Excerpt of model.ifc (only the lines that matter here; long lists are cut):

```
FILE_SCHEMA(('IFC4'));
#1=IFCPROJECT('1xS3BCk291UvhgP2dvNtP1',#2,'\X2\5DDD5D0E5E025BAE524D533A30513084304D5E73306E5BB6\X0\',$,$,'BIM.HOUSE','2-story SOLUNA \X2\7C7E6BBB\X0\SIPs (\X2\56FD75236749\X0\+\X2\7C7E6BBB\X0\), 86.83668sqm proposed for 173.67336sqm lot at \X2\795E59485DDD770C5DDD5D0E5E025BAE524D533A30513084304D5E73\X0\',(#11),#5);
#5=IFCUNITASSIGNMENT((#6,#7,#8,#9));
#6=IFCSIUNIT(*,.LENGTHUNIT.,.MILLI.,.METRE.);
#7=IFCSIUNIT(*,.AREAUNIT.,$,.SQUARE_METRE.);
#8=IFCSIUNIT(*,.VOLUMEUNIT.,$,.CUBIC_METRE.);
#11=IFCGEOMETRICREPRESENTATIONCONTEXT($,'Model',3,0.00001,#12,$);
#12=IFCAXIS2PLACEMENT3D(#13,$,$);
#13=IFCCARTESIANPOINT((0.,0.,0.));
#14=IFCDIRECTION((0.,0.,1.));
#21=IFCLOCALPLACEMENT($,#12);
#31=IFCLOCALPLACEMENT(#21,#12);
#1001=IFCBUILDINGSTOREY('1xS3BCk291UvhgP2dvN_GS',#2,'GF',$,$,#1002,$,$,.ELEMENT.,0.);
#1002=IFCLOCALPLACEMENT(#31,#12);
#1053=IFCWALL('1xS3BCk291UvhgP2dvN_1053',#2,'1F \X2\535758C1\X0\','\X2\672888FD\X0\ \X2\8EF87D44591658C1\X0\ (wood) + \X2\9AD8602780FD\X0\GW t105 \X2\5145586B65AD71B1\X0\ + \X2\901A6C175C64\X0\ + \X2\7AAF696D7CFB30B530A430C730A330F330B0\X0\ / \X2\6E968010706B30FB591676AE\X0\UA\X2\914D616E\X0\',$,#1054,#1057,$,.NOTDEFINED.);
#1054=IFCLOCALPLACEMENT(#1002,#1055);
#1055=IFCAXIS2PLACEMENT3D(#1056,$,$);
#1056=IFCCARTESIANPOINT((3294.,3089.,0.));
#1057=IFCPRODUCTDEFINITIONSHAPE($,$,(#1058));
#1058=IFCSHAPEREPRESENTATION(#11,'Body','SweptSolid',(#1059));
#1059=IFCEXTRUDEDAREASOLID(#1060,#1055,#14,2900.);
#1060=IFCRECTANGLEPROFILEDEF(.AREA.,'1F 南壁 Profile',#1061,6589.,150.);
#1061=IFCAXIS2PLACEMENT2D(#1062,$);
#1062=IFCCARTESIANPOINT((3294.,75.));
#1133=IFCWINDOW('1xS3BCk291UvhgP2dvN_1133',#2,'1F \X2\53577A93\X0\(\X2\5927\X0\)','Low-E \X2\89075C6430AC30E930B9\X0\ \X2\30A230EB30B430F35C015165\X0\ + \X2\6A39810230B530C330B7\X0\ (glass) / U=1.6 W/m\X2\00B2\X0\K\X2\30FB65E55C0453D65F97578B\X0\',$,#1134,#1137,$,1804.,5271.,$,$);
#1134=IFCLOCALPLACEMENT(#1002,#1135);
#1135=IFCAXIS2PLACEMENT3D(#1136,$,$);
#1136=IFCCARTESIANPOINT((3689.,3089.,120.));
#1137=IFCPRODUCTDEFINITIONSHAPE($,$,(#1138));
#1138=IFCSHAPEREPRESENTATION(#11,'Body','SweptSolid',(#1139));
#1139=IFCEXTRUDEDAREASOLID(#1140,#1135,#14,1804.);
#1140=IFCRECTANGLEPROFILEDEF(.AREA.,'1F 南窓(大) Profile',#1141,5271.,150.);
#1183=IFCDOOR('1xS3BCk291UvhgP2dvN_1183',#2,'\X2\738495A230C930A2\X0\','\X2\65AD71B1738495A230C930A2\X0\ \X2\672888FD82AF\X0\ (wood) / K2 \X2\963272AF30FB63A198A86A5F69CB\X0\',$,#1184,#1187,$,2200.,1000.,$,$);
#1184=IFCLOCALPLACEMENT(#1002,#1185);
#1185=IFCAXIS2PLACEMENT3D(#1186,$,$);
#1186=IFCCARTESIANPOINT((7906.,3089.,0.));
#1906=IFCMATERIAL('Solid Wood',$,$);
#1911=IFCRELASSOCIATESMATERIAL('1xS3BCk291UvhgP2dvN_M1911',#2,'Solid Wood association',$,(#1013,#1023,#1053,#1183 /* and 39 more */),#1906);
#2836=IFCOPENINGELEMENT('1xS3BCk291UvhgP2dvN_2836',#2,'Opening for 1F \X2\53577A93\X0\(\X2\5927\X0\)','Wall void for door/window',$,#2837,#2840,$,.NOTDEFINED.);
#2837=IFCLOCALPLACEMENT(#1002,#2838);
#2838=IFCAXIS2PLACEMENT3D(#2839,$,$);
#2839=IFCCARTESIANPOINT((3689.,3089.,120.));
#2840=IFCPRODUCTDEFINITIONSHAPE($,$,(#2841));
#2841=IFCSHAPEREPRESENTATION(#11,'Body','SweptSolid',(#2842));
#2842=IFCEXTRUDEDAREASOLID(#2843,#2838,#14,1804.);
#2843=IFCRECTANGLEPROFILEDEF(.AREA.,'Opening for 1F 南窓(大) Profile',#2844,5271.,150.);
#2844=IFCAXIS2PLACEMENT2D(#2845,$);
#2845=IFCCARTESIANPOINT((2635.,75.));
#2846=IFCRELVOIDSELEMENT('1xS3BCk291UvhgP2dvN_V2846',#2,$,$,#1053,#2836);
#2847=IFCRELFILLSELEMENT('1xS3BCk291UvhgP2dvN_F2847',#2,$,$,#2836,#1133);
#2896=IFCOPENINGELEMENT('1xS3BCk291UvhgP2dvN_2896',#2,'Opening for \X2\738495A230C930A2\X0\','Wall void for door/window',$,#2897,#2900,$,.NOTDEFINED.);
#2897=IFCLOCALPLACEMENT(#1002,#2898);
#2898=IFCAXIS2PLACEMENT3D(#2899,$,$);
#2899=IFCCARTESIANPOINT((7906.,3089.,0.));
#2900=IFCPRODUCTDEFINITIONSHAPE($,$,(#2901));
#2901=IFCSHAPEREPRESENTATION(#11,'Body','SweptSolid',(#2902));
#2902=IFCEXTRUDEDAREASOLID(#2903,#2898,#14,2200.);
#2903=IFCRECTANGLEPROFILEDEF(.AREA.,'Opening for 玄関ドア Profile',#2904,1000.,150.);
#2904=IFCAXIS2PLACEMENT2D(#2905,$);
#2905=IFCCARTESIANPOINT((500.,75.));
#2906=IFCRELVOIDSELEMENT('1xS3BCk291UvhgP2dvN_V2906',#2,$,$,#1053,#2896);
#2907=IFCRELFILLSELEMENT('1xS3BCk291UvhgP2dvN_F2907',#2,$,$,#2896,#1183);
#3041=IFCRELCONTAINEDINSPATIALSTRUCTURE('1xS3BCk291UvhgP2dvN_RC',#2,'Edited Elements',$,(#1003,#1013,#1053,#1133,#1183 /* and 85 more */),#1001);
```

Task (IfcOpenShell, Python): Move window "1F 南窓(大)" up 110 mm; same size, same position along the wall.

```python
import numpy as np
import ifcopenshell
import ifcopenshell.api.geometry
import ifcopenshell.util.placement
import ifcopenshell.util.unit

model = ifcopenshell.open("model.ifc")
unit_scale = ifcopenshell.util.unit.calculate_unit_scale(model)

window = model.by_guid("1xS3BCk291UvhgP2dvN_1133")
opening = window.FillsVoids[0].RelatingOpeningElement
dz = 0.11 / unit_scale

shift = np.array([0.0, 0.0, dz])
# The window is not placed relative to its opening, so move both.
for product in (opening, window):
    matrix = ifcopenshell.util.placement.get_local_placement(product.ObjectPlacement)
    matrix[:3, 3] += shift
    ifcopenshell.api.geometry.edit_object_placement(model, product=product, matrix=matrix, is_si=False)

print(f"moved by {dz * unit_scale:+.3f} m")

model.write("model-out.ifc")
```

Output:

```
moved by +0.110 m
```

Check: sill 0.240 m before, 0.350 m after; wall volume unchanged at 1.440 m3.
